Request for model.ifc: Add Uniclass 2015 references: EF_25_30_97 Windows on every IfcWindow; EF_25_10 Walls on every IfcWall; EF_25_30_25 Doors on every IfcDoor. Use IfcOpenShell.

First a look at what the model holds.

```python
import ifcopenshell

model = ifcopenshell.open("model.ifc")
print(model.schema)
print("classifications:", [c.Name for c in model.by_type("IfcClassification")])
for ifc_class in ("IfcDoor", "IfcRoof", "IfcStair", "IfcWall", "IfcWindow"):
    print(ifc_class, len(model.by_type(ifc_class)))
```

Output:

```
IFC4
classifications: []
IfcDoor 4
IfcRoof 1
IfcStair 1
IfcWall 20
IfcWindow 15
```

```python
import ifcopenshell
import ifcopenshell.api.classification

model = ifcopenshell.open("model.ifc")

system = ifcopenshell.api.classification.add_classification(model, classification="Uniclass 2015")

codes = {
    "IfcWindow": ("EF_25_30_97", "Windows"),
    "IfcWall": ("EF_25_10", "Walls"),
    "IfcDoor": ("EF_25_30_25", "Doors"),
}
for ifc_class, (code, name) in codes.items():
    products = model.by_type(ifc_class)
    ifcopenshell.api.classification.add_reference(
        model, products=products, classification=system, identification=code, name=name
    )
    print(code, len(products))

model.write("model_v2.ifc")
```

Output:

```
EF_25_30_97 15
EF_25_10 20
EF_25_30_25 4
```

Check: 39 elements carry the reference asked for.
